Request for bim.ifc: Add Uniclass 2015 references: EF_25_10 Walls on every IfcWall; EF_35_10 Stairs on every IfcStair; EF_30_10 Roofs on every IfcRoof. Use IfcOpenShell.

First a look at what the model holds.

```python
import ifcopenshell

model = ifcopenshell.open("bim.ifc")
print(model.schema)
print("classifications:", [c.Name for c in model.by_type("IfcClassification")])
for ifc_class in ("IfcDoor", "IfcRoof", "IfcStair", "IfcWall", "IfcWindow"):
    print(ifc_class, len(model.by_type(ifc_class)))
```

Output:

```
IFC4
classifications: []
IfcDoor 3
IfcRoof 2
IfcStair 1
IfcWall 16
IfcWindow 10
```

```python
import ifcopenshell
import ifcopenshell.api.classification

model = ifcopenshell.open("bim.ifc")

system = ifcopenshell.api.classification.add_classification(model, classification="Uniclass 2015")

codes = {
    "IfcWall": ("EF_25_10", "Walls"),
    "IfcStair": ("EF_35_10", "Stairs"),
    "IfcRoof": ("EF_30_10", "Roofs"),
}
for ifc_class, (code, name) in codes.items():
    products = model.by_type(ifc_class)
    ifcopenshell.api.classification.add_reference(
        model, products=products, classification=system, identification=code, name=name
    )
    print(code, len(products))

model.write("bim_v2.ifc")
```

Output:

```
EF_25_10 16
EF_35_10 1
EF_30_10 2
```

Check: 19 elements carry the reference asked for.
